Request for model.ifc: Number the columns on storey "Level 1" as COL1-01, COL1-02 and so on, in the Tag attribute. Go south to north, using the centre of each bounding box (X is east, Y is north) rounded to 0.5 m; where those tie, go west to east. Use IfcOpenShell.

First a look at what the model holds.

```python
import ifcopenshell
import ifcopenshell.util.element
import ifcopenshell.util.placement

model = ifcopenshell.open("model.ifc")
print(model.schema)
storey = next(s for s in model.by_type("IfcBuildingStorey") if s.Name == "Level 1")
columns = [e for e in ifcopenshell.util.element.get_decomposition(storey) if e.is_a("IfcColumn")]
for e in sorted(columns, key=lambda e: e.id()):
    origin = ifcopenshell.util.placement.get_local_placement(e.ObjectPlacement)[:3, 3]
    print(e.id(), e.Tag, e.Name, origin.round(2) + 0.0, sep=" | ")
```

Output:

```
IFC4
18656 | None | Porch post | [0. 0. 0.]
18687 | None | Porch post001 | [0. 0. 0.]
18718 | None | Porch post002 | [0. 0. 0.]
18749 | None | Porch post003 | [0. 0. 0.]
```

```python
import ifcopenshell
import ifcopenshell.geom
import ifcopenshell.util.element
import ifcopenshell.util.shape

model = ifcopenshell.open("model.ifc")
settings = ifcopenshell.geom.settings()
settings.set("use-world-coords", True)


def centre(element):
    shape = ifcopenshell.geom.create_shape(settings, element)
    return ifcopenshell.util.shape.get_bbox_centroid(shape.geometry)


storey = next(s for s in model.by_type("IfcBuildingStorey") if s.Name == "Level 1")
columns = [e for e in ifcopenshell.util.element.get_decomposition(storey) if e.is_a("IfcColumn")]

# Insertion points can sit at a corner or the storey origin, so sort by the geometry (in metres).
centres = {e: centre(e) for e in columns}
columns.sort(key=lambda e: (round(centres[e][1] / 0.5), centres[e][0]))

for i, e in enumerate(columns, start=1):
    number = f"COL1-{i:02d}"
    e.Tag = number
    print(e.id(), number)

model.write("model-out.ifc")
```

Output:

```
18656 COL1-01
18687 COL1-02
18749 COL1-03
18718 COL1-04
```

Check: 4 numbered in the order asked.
